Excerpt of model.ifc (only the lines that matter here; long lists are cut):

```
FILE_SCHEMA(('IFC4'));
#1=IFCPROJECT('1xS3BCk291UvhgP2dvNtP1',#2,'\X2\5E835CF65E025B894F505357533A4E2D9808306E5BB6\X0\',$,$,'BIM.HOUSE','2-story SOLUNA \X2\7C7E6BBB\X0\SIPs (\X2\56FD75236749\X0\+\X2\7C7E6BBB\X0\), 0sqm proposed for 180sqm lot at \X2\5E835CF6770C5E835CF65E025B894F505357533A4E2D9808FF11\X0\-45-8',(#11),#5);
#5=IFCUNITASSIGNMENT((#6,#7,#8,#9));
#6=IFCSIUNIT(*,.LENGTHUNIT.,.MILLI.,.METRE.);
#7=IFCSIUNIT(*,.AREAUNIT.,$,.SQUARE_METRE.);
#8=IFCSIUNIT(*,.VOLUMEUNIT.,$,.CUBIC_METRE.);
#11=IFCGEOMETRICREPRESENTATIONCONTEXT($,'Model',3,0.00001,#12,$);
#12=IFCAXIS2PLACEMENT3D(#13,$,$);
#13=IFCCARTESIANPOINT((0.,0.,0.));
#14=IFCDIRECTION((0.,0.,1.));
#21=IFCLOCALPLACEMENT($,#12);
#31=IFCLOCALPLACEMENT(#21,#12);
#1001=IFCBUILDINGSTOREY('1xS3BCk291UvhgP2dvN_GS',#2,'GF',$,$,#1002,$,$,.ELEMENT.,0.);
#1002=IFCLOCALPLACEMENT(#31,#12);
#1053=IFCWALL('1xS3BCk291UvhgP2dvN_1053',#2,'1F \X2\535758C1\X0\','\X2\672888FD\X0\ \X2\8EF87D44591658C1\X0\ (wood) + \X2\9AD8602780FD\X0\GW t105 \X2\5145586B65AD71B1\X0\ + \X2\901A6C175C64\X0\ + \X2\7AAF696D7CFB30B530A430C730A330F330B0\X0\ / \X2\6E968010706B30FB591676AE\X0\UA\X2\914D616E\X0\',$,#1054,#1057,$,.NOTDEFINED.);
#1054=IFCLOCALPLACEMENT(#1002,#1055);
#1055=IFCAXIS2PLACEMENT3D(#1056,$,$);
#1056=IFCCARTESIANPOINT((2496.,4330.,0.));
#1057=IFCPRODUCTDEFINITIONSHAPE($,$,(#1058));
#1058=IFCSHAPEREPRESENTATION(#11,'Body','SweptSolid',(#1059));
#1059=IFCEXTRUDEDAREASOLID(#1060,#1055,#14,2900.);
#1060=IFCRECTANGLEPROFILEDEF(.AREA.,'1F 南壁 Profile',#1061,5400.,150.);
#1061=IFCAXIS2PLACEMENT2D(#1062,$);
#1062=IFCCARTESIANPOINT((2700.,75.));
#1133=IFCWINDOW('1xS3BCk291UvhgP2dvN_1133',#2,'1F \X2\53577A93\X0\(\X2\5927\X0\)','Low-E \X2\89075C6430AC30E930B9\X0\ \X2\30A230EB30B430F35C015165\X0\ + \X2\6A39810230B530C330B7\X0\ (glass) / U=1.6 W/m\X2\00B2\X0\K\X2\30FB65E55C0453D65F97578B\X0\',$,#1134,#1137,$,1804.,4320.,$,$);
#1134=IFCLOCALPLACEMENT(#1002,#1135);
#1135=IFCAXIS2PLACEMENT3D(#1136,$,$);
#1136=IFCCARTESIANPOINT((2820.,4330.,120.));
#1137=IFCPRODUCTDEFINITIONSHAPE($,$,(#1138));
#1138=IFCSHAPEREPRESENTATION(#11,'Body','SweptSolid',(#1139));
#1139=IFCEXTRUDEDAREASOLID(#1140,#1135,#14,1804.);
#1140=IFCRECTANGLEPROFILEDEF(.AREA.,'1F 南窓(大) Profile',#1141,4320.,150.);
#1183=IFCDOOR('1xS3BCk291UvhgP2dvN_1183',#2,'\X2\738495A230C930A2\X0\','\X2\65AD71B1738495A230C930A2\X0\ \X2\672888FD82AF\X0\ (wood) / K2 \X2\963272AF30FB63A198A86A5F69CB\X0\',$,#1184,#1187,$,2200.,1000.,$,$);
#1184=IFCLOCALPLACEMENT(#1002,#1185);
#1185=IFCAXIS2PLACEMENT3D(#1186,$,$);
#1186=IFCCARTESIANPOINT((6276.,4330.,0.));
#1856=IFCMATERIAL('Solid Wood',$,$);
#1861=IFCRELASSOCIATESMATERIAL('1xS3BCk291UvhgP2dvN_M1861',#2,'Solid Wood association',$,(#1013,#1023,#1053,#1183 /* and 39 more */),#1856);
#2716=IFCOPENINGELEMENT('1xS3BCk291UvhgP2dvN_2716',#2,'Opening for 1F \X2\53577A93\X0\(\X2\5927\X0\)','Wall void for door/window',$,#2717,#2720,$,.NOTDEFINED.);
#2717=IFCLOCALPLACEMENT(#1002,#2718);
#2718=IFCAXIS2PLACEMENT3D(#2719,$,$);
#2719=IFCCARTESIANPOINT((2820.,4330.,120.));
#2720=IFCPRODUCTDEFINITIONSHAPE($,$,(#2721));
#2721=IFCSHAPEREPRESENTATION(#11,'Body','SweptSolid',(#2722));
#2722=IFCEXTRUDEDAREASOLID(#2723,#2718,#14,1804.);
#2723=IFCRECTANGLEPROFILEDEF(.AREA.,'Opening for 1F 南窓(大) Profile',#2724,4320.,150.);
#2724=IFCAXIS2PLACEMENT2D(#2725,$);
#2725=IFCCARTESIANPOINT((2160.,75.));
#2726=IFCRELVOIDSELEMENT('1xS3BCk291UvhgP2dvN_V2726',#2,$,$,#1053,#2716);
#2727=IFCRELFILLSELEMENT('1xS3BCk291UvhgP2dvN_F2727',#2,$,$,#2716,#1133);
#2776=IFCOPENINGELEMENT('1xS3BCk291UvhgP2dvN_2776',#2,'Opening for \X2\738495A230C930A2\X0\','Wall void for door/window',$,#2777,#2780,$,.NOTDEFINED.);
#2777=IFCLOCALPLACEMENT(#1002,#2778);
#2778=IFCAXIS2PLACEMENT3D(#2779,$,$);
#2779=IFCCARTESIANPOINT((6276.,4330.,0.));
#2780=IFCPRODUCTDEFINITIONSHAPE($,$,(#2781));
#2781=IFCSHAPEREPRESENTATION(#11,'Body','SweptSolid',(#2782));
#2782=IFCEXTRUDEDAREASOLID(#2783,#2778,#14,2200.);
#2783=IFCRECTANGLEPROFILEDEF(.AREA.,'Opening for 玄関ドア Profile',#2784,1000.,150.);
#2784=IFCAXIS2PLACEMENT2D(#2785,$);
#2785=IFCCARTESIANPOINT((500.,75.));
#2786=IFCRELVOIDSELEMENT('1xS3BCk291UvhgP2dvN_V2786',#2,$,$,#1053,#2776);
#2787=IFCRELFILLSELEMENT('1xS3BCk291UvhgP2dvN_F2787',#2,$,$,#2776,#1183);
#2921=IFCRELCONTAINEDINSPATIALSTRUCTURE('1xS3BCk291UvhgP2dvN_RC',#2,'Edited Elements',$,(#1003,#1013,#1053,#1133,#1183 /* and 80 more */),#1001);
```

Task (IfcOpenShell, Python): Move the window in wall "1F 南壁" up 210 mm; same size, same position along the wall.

```python
import numpy as np
import ifcopenshell
import ifcopenshell.api.geometry
import ifcopenshell.util.placement
import ifcopenshell.util.unit

model = ifcopenshell.open("model.ifc")
unit_scale = ifcopenshell.util.unit.calculate_unit_scale(model)

window = model.by_guid("1xS3BCk291UvhgP2dvN_1133")
opening = window.FillsVoids[0].RelatingOpeningElement
dz = 210.0

shift = np.array([0.0, 0.0, dz])
# The window is not placed relative to its opening, so move both.
for product in (opening, window):
    matrix = ifcopenshell.util.placement.get_local_placement(product.ObjectPlacement)
    matrix[:3, 3] += shift
    ifcopenshell.api.geometry.edit_object_placement(model, product=product, matrix=matrix, is_si=False)

print(f"moved by {dz * unit_scale:+.3f} m")

model.write("model_updated.ifc")
```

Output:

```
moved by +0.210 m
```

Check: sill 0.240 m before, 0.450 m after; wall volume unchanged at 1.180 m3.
